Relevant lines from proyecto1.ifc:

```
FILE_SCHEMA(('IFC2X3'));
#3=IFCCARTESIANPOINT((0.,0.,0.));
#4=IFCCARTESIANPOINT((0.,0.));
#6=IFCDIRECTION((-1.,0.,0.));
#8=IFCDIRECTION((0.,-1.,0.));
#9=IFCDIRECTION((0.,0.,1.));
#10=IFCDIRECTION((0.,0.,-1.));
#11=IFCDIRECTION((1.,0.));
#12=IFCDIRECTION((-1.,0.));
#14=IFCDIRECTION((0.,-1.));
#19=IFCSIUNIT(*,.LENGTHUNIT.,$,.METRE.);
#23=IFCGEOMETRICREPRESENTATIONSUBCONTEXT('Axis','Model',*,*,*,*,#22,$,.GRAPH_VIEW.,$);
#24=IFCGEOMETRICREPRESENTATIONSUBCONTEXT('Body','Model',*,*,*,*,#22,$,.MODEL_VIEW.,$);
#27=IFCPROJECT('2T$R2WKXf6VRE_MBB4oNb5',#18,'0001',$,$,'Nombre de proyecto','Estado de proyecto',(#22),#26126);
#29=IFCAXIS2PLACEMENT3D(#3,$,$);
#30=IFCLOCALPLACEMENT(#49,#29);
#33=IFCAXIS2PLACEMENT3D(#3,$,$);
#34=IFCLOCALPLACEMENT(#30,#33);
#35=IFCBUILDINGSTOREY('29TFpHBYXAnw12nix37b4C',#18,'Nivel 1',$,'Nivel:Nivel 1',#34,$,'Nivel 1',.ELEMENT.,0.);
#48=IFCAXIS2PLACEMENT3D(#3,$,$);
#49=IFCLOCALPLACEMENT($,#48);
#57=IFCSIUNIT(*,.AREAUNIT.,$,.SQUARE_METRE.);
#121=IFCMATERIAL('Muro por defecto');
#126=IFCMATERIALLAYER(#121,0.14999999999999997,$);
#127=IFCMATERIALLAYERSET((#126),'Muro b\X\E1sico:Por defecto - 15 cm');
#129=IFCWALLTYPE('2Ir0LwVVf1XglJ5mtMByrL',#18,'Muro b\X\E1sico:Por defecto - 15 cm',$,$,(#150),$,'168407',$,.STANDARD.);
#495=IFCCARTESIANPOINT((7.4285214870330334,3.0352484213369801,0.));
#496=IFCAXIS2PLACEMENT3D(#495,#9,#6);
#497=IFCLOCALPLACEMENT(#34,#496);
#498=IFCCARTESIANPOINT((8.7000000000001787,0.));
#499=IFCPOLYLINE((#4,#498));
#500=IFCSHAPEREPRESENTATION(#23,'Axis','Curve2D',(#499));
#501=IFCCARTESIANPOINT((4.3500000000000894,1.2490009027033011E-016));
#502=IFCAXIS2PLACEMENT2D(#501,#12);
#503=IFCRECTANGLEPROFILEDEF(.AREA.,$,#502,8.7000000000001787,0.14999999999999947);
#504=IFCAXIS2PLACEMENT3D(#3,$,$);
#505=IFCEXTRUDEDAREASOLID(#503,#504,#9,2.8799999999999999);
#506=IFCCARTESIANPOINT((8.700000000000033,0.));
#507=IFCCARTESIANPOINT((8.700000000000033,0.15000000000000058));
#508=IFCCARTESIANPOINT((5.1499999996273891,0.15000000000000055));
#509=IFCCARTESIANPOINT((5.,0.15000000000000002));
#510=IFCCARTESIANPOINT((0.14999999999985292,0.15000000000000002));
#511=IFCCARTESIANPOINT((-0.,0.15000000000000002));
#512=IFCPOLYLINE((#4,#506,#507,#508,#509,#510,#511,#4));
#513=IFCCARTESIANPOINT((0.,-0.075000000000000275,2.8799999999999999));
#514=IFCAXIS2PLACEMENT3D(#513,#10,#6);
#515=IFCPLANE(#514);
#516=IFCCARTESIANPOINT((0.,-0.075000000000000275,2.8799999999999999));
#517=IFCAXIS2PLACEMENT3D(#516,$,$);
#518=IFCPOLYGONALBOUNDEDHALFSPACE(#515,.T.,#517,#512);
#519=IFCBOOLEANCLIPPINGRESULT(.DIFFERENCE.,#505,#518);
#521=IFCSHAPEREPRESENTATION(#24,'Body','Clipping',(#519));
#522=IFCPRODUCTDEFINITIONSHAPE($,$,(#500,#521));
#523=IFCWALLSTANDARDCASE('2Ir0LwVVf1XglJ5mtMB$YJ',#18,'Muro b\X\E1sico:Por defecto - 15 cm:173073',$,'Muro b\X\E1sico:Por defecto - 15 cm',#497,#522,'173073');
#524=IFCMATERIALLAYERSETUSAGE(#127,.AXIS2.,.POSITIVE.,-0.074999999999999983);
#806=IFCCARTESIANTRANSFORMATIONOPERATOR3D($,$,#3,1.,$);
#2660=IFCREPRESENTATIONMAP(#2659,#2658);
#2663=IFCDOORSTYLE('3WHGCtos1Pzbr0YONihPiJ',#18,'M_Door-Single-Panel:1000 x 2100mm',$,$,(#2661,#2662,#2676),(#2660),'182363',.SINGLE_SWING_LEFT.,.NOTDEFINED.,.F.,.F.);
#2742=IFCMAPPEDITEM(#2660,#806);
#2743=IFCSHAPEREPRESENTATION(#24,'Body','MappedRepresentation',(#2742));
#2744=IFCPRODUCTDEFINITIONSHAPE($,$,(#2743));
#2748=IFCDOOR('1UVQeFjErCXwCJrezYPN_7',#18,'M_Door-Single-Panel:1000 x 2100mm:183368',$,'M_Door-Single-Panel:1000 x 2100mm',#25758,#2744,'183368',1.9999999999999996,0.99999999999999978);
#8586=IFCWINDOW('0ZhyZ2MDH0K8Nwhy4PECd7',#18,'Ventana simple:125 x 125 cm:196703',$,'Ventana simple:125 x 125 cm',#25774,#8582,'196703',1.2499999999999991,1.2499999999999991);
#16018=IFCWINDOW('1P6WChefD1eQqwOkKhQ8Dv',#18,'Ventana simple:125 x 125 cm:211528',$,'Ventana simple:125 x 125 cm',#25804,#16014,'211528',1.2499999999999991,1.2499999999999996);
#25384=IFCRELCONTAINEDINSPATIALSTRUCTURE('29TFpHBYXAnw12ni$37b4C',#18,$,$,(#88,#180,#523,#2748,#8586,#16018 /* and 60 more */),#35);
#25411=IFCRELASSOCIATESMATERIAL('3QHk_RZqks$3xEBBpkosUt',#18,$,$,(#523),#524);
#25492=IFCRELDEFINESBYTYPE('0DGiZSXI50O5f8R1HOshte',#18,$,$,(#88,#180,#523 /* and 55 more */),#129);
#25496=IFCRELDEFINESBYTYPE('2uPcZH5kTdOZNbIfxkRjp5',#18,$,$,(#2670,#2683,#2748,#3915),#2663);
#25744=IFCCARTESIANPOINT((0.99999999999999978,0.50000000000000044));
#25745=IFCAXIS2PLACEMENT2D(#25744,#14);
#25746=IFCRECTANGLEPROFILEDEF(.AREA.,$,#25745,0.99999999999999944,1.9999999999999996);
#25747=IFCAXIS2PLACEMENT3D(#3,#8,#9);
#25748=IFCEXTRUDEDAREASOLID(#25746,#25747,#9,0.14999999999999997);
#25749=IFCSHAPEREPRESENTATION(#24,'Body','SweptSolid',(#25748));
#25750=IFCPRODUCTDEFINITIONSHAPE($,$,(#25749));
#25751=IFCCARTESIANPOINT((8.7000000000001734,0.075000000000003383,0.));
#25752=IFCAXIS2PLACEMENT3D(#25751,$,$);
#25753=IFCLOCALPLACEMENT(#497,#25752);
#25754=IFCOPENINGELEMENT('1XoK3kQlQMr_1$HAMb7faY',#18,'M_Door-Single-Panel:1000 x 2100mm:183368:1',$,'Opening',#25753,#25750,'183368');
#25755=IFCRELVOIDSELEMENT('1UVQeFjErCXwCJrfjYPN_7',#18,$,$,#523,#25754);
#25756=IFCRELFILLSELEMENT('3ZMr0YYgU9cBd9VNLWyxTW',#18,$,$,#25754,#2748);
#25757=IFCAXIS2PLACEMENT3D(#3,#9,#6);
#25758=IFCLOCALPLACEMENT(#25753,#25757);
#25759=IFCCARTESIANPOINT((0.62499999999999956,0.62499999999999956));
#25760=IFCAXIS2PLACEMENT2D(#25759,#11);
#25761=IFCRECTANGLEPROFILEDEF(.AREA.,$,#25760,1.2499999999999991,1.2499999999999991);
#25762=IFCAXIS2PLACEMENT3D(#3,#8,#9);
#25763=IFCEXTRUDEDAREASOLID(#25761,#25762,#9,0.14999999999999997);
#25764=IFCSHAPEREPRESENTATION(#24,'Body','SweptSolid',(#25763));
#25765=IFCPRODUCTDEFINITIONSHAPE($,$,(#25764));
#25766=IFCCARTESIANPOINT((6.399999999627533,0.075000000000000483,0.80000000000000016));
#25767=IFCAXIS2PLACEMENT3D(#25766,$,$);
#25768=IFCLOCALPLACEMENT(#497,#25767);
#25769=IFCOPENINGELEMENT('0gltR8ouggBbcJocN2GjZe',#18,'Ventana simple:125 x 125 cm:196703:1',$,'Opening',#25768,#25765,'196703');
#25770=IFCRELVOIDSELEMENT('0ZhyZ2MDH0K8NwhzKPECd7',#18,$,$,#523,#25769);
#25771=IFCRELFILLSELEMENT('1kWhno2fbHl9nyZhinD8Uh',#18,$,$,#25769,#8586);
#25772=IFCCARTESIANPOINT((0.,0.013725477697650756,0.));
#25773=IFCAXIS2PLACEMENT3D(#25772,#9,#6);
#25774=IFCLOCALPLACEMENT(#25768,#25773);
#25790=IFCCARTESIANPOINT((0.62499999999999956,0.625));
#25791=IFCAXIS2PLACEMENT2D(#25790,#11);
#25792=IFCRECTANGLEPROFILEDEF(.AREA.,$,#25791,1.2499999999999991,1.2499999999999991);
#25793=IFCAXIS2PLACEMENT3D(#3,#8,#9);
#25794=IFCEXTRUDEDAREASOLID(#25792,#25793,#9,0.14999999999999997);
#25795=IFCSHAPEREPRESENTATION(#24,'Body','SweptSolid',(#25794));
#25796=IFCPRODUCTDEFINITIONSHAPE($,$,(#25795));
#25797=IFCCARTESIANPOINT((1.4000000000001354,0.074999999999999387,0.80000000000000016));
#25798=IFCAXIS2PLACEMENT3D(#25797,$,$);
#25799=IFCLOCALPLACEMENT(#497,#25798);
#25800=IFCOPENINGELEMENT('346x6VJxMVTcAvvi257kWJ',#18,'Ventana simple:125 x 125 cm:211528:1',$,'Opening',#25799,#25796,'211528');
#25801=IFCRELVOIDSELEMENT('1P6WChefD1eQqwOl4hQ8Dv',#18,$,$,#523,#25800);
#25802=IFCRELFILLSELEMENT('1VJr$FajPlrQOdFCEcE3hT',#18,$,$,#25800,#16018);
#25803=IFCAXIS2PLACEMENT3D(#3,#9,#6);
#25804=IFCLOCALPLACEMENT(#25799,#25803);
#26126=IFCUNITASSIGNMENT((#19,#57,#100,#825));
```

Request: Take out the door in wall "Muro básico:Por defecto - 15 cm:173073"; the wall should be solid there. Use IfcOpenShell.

```python
import ifcopenshell
import ifcopenshell.api.feature
import ifcopenshell.api.root
import ifcopenshell.geom
import ifcopenshell.util.shape

model = ifcopenshell.open("proyecto1.ifc")
settings = ifcopenshell.geom.settings()


def volume(element):
    """Net volume in cubic metres, openings subtracted."""
    shape = ifcopenshell.geom.create_shape(settings, element)
    return ifcopenshell.util.shape.get_volume(shape.geometry)


door = model.by_guid("1UVQeFjErCXwCJrezYPN_7")
opening = door.FillsVoids[0].RelatingOpeningElement
wall = opening.VoidsElements[0].RelatingBuildingElement
before = volume(wall)

ifcopenshell.api.root.remove_product(model, product=door)
ifcopenshell.api.feature.remove_feature(model, feature=opening)

after = volume(wall)

print(f"wall volume {before:.3f} -> {after:.3f} m3")

model.write("proyecto1_updated.ifc")
```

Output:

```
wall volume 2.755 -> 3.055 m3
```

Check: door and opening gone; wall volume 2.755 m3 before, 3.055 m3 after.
